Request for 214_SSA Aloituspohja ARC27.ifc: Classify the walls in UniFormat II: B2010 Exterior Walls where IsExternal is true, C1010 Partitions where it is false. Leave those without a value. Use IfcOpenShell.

First a look at what the model holds.

```python
import ifcopenshell
import ifcopenshell.util.element

model = ifcopenshell.open("214_SSA Aloituspohja ARC27.ifc")
print(model.schema)
print("classifications:", [c.Name for c in model.by_type("IfcClassification")])
values = [ifcopenshell.util.element.get_pset(e, "Pset_WallCommon", "IsExternal") for e in model.by_type("IfcWall")]
for value in (True, False, None):
    print("IsExternal", value, values.count(value))
```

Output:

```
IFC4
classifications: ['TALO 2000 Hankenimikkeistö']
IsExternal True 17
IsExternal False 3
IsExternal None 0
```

```python
import ifcopenshell
import ifcopenshell.api.classification
import ifcopenshell.util.element

model = ifcopenshell.open("214_SSA Aloituspohja ARC27.ifc")

system = ifcopenshell.api.classification.add_classification(model, classification="UniFormat II")

walls = model.by_type("IfcWall")
external = {e: ifcopenshell.util.element.get_pset(e, "Pset_WallCommon", "IsExternal") for e in walls}
for flag, code, name in ((True, "B2010", "Exterior Walls"), (False, "C1010", "Partitions")):
    products = [e for e in walls if external[e] is flag]
    ifcopenshell.api.classification.add_reference(
        model, products=products, classification=system, identification=code, name=name
    )
    print(code, len(products))

model.write("214_SSA Aloituspohja ARC27_updated.ifc")
```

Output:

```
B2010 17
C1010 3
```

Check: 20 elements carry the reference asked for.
